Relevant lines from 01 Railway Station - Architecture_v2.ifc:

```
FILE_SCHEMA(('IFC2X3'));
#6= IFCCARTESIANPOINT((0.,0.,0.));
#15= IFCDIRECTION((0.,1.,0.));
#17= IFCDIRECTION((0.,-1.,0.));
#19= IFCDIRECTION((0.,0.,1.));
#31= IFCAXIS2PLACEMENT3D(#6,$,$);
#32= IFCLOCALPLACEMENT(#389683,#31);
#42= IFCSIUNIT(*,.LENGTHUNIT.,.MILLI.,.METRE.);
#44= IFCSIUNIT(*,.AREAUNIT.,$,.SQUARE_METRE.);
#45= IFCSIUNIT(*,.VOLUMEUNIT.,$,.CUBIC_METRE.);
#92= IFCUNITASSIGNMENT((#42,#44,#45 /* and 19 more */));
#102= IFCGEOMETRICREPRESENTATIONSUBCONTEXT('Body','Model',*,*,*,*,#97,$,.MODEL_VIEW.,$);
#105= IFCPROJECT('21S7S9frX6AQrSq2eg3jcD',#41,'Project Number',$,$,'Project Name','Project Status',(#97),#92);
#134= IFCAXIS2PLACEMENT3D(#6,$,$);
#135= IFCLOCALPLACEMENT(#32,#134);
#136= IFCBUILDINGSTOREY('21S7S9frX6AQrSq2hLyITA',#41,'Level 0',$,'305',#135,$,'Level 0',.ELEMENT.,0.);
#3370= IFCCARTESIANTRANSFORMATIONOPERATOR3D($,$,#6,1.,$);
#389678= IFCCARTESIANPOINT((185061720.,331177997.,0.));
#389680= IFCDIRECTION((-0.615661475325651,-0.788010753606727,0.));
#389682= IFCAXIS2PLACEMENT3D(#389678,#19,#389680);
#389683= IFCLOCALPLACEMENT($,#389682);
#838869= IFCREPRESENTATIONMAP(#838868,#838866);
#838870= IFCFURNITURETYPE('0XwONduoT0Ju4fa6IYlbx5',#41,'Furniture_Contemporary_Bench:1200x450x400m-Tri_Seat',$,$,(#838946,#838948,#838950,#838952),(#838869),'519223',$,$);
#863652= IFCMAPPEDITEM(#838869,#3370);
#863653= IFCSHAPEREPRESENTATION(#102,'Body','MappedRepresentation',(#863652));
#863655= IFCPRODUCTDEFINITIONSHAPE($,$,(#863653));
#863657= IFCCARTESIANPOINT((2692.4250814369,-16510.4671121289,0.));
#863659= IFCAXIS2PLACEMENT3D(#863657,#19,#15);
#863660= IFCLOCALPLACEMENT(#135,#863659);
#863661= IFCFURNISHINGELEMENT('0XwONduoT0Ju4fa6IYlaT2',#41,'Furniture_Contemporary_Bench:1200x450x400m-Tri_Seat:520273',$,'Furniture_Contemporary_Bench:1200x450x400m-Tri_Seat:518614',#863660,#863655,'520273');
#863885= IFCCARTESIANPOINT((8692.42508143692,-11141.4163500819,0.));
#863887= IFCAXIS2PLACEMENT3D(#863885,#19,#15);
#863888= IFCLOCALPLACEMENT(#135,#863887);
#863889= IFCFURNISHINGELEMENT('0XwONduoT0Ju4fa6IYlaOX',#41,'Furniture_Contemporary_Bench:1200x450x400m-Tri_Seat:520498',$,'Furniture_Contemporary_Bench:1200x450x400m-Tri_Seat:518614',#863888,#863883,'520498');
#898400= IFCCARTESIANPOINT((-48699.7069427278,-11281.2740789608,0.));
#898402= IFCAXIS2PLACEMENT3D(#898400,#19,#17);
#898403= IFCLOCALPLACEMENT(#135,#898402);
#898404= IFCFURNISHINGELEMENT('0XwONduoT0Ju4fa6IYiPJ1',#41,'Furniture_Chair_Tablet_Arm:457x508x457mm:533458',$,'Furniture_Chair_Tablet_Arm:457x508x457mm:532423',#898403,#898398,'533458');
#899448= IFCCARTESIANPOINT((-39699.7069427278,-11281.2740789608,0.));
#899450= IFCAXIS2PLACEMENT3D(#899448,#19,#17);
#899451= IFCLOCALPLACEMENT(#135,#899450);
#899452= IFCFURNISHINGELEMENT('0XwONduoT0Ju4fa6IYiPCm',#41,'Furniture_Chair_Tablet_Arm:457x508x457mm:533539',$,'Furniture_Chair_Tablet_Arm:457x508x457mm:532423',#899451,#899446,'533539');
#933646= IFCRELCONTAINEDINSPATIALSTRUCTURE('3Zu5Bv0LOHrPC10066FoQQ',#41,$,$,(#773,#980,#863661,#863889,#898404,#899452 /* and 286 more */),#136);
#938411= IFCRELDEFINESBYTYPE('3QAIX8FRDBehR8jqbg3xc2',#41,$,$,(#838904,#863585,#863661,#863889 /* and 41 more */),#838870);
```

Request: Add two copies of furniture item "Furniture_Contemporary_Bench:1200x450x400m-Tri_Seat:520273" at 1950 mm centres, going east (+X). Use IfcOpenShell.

```python
import numpy as np
import ifcopenshell
import ifcopenshell.api.geometry
import ifcopenshell.api.root
import ifcopenshell.util.element
import ifcopenshell.util.placement
import ifcopenshell.util.unit

model = ifcopenshell.open("01 Railway Station - Architecture_v2.ifc")
unit_scale = ifcopenshell.util.unit.calculate_unit_scale(model)


def reuse_history(source, copy):
    """copy_class also copies each property set's owner history, people and application; keep the originals."""
    for rel in copy.IsDefinedBy:
        if rel.is_a("IfcRelDefinesByProperties") and (history := rel.RelatingPropertyDefinition.OwnerHistory):
            rel.RelatingPropertyDefinition.OwnerHistory = source.OwnerHistory
            ifcopenshell.util.element.remove_deep2(model, history)


source = model.by_guid("0XwONduoT0Ju4fa6IYlaT2")
base = ifcopenshell.util.placement.get_local_placement(source.ObjectPlacement)
step = np.array([1.0, 0.0, 0.0]) * 1.95 / unit_scale

for i in range(1, 3):
    copy = ifcopenshell.api.root.copy_class(model, product=source)
    copy.Representation = ifcopenshell.util.element.copy_deep(
        model, source.Representation, exclude=["IfcGeometricRepresentationContext", "IfcRepresentationMap"]
    )
    copy.Name = "Furniture_Contemporary_Bench:1200x450x400m-Tri_Seat"
    copy.Tag = None
    reuse_history(source, copy)
    matrix = base.copy()
    matrix[:3, 3] += i * step
    print("added at", matrix[:3, 3].round(3) + 0.0)
    ifcopenshell.api.geometry.edit_object_placement(model, product=copy, matrix=matrix, is_si=False)

model.write("01 Railway Station - Architecture_v2_updated.ifc")
```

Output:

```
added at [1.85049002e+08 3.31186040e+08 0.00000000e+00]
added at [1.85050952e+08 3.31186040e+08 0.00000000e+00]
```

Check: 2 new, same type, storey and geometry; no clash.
